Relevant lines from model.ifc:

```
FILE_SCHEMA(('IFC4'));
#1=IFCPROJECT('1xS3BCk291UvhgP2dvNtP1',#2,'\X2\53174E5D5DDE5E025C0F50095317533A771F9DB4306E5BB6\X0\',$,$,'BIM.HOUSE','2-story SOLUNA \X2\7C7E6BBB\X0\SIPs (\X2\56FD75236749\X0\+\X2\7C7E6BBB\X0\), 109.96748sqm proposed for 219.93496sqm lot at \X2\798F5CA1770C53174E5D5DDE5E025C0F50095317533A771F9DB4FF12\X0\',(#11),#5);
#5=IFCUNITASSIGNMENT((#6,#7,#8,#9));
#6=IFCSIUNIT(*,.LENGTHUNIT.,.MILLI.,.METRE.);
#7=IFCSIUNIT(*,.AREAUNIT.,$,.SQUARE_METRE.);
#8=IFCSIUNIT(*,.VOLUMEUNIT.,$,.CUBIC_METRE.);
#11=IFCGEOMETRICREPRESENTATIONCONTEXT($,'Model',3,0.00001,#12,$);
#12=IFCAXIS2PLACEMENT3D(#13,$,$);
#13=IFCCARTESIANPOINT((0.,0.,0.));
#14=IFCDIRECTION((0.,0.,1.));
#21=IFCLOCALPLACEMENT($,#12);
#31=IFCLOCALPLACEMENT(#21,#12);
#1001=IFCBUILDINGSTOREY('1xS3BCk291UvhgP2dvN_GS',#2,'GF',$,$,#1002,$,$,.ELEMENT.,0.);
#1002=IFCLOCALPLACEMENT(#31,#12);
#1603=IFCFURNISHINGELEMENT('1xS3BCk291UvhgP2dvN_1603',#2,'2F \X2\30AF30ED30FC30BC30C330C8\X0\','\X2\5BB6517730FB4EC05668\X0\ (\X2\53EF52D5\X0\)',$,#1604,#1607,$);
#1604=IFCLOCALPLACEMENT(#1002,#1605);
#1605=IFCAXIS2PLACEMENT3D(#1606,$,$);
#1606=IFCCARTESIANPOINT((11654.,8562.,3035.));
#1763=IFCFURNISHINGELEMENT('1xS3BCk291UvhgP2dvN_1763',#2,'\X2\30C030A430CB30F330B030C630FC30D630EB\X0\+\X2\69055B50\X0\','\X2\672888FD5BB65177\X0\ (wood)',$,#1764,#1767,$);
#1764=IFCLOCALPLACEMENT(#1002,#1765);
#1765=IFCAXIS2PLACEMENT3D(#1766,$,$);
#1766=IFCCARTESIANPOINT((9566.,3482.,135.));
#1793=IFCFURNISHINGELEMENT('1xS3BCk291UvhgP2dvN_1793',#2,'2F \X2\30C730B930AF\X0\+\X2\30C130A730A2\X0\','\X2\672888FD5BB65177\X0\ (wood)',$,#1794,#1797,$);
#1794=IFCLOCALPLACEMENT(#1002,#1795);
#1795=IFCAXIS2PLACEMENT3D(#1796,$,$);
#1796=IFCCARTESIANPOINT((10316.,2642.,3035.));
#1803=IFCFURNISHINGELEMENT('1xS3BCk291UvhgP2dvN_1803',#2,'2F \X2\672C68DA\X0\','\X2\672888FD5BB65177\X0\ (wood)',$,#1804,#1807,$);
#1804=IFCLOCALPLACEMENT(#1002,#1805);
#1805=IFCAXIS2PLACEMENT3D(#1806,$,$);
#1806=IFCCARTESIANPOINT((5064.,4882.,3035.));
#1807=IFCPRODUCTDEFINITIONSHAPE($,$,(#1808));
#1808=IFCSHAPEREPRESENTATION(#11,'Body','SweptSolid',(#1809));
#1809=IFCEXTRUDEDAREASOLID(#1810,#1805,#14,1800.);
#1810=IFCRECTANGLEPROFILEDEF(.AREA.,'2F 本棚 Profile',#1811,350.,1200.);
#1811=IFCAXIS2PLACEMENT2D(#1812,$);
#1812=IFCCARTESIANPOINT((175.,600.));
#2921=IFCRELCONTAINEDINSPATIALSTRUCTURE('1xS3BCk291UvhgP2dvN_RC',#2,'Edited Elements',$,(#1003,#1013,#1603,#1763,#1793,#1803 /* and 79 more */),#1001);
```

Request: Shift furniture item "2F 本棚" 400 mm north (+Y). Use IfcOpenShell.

```python
import ifcopenshell
import ifcopenshell.api.geometry
import ifcopenshell.util.placement
import ifcopenshell.util.unit

model = ifcopenshell.open("model.ifc")
unit_scale = ifcopenshell.util.unit.calculate_unit_scale(model)

item = model.by_guid("1xS3BCk291UvhgP2dvN_1803")
matrix = ifcopenshell.util.placement.get_local_placement(item.ObjectPlacement)
matrix[1, 3] += 0.4 / unit_scale
ifcopenshell.api.geometry.edit_object_placement(model, product=item, matrix=matrix, is_si=False)

print(ifcopenshell.util.placement.get_local_placement(item.ObjectPlacement).round(3) + 0.0)

model.write("model_edited.ifc")
```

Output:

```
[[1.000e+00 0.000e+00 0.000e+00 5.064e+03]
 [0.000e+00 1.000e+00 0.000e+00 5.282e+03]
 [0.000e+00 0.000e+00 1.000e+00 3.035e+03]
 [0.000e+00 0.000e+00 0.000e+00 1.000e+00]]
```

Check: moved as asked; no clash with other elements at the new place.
